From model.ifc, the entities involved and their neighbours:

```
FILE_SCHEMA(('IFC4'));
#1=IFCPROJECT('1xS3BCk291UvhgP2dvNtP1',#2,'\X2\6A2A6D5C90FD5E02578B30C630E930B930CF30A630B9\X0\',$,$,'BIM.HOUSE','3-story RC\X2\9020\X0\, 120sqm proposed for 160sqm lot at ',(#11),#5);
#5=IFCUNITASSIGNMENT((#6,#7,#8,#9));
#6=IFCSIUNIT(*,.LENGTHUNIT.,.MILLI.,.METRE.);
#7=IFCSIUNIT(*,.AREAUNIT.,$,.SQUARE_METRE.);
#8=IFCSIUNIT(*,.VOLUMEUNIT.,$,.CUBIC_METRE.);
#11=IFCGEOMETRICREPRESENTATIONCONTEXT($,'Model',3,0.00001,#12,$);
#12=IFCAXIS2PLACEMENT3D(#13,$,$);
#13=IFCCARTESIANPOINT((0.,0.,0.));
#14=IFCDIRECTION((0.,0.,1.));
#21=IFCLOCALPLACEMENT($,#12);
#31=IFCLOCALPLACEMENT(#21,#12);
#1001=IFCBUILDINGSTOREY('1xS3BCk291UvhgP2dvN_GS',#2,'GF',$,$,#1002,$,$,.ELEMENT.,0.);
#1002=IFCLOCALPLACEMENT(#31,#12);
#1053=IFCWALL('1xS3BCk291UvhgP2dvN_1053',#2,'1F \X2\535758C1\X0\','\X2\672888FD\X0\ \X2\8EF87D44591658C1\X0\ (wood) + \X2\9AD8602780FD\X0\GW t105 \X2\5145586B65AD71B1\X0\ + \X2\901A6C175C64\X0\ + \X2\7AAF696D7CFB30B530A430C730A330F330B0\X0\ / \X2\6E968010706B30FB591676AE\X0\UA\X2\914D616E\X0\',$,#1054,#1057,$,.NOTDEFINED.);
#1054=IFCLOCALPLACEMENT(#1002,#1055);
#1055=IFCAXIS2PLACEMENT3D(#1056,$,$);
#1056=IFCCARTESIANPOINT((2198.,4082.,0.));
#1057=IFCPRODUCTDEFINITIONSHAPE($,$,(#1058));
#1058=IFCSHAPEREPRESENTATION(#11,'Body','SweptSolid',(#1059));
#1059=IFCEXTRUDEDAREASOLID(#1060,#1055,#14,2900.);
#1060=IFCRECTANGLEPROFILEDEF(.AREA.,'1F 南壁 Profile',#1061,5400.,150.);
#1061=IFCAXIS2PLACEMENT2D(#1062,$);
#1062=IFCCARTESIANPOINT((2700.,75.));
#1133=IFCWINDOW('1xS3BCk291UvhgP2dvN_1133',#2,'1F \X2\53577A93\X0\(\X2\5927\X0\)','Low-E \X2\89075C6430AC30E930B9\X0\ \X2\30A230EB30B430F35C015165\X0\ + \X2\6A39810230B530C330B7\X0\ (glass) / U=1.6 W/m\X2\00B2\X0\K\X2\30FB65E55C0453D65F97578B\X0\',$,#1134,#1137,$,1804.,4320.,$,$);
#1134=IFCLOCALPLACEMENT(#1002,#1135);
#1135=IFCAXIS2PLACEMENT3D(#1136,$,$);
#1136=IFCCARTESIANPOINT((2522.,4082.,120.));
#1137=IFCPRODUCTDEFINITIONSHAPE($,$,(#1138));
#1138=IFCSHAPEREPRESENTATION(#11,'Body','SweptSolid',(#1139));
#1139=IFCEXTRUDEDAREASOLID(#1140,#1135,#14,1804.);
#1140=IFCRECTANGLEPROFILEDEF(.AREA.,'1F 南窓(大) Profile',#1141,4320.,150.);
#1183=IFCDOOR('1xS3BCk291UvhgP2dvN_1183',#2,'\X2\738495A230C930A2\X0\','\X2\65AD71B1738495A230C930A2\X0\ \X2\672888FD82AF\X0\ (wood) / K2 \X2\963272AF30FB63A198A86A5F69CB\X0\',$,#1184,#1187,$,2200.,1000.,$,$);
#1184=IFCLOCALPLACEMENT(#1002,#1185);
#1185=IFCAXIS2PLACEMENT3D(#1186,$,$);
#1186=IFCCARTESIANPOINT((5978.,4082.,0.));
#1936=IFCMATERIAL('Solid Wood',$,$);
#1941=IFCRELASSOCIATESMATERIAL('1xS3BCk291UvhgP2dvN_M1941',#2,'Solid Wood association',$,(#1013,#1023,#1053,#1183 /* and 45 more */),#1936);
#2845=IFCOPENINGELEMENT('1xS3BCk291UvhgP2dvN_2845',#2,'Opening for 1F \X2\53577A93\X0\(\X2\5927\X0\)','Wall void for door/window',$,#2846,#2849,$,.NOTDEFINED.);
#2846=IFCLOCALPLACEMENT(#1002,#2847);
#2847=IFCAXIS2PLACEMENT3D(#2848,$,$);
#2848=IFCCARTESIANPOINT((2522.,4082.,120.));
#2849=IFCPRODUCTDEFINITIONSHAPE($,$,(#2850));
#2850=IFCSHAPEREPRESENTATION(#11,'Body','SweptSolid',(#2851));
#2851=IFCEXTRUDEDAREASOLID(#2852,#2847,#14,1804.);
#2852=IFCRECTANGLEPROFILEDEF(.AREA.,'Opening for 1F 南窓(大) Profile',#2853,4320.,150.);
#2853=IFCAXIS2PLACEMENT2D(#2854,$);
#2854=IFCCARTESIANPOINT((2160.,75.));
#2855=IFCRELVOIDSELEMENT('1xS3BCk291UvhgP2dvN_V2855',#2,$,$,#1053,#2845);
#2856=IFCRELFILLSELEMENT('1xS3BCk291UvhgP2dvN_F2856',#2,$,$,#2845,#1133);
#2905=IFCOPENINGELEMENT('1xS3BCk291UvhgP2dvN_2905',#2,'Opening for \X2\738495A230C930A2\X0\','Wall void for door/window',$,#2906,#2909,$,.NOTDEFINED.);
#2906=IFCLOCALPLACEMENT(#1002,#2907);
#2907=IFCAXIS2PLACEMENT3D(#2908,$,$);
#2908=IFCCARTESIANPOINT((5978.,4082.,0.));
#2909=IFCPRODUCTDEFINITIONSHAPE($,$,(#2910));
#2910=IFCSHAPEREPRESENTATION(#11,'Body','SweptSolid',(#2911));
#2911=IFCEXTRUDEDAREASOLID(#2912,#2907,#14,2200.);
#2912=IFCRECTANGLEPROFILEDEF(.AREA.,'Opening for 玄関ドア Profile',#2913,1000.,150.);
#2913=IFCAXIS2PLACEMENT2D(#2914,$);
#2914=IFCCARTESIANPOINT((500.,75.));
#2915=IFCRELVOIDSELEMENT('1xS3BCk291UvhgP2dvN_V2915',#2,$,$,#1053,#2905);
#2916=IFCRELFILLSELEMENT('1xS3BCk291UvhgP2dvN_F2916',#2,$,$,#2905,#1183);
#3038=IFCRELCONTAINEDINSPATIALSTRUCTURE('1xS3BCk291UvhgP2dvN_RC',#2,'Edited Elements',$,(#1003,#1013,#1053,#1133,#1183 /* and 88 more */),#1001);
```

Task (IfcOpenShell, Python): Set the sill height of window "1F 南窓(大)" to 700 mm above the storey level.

```python
import numpy as np
import ifcopenshell
import ifcopenshell.api.geometry
import ifcopenshell.geom
import ifcopenshell.util.element
import ifcopenshell.util.placement
import ifcopenshell.util.shape
import ifcopenshell.util.unit

model = ifcopenshell.open("model.ifc")
unit_scale = ifcopenshell.util.unit.calculate_unit_scale(model)

window = model.by_guid("1xS3BCk291UvhgP2dvN_1133")
opening = window.FillsVoids[0].RelatingOpeningElement
storey = ifcopenshell.util.element.get_container(window, ifc_class="IfcBuildingStorey")
level = ifcopenshell.util.placement.get_local_placement(storey.ObjectPlacement)[2, 3]

# The opening's origin need not be at the sill, so measure its lowest point.
shape = ifcopenshell.geom.create_shape(ifcopenshell.geom.settings(), opening)
bottom = ifcopenshell.util.shape.get_shape_bottom_elevation(shape, shape.geometry) / unit_scale
dz = level + 0.7 / unit_scale - bottom

shift = np.array([0.0, 0.0, dz])
# The window is not placed relative to its opening, so move both.
for product in (opening, window):
    matrix = ifcopenshell.util.placement.get_local_placement(product.ObjectPlacement)
    matrix[:3, 3] += shift
    ifcopenshell.api.geometry.edit_object_placement(model, product=product, matrix=matrix, is_si=False)

print(f"moved by {dz * unit_scale:+.3f} m")

model.write("model-out.ifc")
```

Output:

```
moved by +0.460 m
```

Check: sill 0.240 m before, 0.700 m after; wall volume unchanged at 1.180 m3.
